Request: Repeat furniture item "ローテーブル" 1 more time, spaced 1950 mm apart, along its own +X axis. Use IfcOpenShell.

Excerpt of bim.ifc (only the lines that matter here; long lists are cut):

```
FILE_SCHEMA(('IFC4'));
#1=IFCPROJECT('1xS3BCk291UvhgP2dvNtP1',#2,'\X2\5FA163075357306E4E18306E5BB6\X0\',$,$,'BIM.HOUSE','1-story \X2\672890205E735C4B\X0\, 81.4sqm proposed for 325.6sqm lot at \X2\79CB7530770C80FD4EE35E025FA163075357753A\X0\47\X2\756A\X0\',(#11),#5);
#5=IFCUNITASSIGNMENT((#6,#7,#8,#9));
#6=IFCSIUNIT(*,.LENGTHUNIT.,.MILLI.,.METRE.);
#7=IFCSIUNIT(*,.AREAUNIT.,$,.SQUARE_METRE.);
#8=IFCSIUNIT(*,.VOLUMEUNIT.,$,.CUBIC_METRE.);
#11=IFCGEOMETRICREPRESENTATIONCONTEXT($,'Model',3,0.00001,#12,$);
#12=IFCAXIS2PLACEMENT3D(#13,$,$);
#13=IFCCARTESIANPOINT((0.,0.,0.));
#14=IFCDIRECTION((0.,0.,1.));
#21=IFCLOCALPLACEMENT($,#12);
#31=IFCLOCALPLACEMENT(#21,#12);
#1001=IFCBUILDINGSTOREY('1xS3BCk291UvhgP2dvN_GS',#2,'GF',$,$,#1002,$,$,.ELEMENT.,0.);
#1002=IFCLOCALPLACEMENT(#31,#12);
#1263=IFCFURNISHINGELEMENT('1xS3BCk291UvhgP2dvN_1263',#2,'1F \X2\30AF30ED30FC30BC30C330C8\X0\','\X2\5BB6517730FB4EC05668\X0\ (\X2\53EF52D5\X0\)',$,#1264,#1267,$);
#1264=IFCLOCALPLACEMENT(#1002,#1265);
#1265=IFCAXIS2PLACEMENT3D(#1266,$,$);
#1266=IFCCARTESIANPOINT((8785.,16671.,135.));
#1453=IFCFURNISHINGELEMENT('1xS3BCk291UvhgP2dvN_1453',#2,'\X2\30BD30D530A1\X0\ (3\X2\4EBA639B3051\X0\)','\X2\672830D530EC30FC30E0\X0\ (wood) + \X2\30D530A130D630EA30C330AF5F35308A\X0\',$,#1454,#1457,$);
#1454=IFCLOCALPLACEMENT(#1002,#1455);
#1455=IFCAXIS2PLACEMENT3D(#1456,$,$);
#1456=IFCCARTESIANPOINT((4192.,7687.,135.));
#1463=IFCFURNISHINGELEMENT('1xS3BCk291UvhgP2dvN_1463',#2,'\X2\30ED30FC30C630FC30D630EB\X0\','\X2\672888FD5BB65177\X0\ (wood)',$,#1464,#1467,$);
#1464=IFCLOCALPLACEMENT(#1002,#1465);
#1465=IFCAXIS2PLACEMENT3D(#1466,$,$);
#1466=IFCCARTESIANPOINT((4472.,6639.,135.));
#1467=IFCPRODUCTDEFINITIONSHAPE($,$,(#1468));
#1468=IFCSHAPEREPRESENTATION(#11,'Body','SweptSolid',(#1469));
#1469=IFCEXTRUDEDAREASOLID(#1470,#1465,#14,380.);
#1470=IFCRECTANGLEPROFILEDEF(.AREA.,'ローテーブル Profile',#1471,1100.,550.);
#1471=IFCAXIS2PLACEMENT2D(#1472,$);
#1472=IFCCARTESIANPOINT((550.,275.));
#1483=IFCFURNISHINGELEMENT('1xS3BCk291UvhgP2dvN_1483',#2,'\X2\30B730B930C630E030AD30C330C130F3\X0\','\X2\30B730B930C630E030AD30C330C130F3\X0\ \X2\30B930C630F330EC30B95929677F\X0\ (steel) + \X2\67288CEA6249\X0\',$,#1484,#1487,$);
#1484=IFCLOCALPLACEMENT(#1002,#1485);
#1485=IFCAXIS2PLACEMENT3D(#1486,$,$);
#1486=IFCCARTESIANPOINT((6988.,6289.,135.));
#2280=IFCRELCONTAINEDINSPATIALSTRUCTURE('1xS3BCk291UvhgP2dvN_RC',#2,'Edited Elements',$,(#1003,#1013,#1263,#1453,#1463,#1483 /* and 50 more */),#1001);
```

```python
import ifcopenshell
import ifcopenshell.api.geometry
import ifcopenshell.api.root
import ifcopenshell.util.element
import ifcopenshell.util.placement

model = ifcopenshell.open("bim.ifc")


def reuse_history(source, copy):
    """copy_class also copies each property set's owner history, people and application; keep the originals."""
    for rel in copy.IsDefinedBy:
        if rel.is_a("IfcRelDefinesByProperties") and (history := rel.RelatingPropertyDefinition.OwnerHistory):
            rel.RelatingPropertyDefinition.OwnerHistory = source.OwnerHistory
            ifcopenshell.util.element.remove_deep2(model, history)


source = model.by_guid("1xS3BCk291UvhgP2dvN_1463")
base = ifcopenshell.util.placement.get_local_placement(source.ObjectPlacement)
step = base[:3, 0] * 1950.0

for i in range(1, 2):
    copy = ifcopenshell.api.root.copy_class(model, product=source)
    copy.Representation = ifcopenshell.util.element.copy_deep(
        model, source.Representation, exclude=["IfcGeometricRepresentationContext", "IfcRepresentationMap"]
    )
    reuse_history(source, copy)
    matrix = base.copy()
    matrix[:3, 3] += i * step
    print("added at", matrix[:3, 3].round(3) + 0.0)
    ifcopenshell.api.geometry.edit_object_placement(model, product=copy, matrix=matrix, is_si=False)

model.write("bim_edited.ifc")
```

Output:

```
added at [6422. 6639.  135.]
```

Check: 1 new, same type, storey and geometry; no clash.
